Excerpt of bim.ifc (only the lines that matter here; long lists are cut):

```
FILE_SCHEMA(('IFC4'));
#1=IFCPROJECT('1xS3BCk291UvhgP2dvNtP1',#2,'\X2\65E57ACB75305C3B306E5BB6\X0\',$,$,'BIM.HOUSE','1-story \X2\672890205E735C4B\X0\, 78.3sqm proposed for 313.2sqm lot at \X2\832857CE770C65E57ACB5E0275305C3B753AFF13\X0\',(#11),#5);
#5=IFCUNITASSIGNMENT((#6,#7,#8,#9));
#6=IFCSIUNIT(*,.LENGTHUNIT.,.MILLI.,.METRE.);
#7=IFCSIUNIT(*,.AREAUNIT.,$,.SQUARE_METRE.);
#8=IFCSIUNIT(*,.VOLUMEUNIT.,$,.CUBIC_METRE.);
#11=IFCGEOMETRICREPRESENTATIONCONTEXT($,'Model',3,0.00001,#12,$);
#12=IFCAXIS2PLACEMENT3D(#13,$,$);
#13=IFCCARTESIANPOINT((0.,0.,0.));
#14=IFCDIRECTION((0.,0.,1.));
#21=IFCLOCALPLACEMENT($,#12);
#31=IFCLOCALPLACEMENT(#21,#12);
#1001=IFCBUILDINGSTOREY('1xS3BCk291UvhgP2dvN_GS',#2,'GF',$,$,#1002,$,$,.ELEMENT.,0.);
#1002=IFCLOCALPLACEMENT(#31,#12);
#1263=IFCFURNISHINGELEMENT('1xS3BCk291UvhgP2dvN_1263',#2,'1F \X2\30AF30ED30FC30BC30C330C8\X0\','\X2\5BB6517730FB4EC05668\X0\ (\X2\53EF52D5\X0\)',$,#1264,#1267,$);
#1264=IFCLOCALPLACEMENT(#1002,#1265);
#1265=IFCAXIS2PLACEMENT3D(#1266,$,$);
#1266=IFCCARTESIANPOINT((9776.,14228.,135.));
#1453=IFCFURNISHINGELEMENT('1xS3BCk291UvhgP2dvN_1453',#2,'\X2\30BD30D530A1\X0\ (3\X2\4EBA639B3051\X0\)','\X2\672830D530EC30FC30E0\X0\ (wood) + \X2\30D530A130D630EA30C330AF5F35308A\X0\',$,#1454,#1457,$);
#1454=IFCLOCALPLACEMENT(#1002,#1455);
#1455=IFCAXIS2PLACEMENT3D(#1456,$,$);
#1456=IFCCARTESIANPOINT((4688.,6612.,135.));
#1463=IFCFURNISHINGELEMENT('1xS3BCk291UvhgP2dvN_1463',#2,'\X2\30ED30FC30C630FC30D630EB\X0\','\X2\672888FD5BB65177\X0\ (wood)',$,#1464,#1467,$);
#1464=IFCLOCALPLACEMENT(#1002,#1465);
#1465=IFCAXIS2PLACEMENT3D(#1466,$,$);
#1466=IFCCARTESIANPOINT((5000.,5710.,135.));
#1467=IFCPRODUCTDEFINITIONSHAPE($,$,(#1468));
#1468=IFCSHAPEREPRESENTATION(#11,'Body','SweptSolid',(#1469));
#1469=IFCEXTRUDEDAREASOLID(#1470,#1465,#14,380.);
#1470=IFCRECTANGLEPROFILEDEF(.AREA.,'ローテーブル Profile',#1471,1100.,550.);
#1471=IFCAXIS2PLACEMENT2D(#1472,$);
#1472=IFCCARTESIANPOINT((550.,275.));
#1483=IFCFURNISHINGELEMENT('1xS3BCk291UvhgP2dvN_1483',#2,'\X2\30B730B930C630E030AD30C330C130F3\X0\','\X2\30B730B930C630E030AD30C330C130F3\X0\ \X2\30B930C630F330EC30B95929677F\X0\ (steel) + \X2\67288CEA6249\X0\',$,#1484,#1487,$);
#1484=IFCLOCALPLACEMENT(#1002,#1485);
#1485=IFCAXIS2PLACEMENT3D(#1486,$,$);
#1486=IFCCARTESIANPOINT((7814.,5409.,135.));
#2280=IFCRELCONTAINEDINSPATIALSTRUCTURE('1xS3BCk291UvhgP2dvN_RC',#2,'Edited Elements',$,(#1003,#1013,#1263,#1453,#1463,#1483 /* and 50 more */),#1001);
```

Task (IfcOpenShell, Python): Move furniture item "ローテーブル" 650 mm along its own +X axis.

```python
import ifcopenshell
import ifcopenshell.api.geometry
import ifcopenshell.util.placement
import ifcopenshell.util.unit

model = ifcopenshell.open("bim.ifc")
unit_scale = ifcopenshell.util.unit.calculate_unit_scale(model)

item = model.by_id(1463)
matrix = ifcopenshell.util.placement.get_local_placement(item.ObjectPlacement)
matrix[:3, 3] += matrix[:3, 0] * 0.65 / unit_scale
ifcopenshell.api.geometry.edit_object_placement(model, product=item, matrix=matrix, is_si=False)

print(ifcopenshell.util.placement.get_local_placement(item.ObjectPlacement).round(3) + 0.0)

model.write("bim_rev.ifc")
```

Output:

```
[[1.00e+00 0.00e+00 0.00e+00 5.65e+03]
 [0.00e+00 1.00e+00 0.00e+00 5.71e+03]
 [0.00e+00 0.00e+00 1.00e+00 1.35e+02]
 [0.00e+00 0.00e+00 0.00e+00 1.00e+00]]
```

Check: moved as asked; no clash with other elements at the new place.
